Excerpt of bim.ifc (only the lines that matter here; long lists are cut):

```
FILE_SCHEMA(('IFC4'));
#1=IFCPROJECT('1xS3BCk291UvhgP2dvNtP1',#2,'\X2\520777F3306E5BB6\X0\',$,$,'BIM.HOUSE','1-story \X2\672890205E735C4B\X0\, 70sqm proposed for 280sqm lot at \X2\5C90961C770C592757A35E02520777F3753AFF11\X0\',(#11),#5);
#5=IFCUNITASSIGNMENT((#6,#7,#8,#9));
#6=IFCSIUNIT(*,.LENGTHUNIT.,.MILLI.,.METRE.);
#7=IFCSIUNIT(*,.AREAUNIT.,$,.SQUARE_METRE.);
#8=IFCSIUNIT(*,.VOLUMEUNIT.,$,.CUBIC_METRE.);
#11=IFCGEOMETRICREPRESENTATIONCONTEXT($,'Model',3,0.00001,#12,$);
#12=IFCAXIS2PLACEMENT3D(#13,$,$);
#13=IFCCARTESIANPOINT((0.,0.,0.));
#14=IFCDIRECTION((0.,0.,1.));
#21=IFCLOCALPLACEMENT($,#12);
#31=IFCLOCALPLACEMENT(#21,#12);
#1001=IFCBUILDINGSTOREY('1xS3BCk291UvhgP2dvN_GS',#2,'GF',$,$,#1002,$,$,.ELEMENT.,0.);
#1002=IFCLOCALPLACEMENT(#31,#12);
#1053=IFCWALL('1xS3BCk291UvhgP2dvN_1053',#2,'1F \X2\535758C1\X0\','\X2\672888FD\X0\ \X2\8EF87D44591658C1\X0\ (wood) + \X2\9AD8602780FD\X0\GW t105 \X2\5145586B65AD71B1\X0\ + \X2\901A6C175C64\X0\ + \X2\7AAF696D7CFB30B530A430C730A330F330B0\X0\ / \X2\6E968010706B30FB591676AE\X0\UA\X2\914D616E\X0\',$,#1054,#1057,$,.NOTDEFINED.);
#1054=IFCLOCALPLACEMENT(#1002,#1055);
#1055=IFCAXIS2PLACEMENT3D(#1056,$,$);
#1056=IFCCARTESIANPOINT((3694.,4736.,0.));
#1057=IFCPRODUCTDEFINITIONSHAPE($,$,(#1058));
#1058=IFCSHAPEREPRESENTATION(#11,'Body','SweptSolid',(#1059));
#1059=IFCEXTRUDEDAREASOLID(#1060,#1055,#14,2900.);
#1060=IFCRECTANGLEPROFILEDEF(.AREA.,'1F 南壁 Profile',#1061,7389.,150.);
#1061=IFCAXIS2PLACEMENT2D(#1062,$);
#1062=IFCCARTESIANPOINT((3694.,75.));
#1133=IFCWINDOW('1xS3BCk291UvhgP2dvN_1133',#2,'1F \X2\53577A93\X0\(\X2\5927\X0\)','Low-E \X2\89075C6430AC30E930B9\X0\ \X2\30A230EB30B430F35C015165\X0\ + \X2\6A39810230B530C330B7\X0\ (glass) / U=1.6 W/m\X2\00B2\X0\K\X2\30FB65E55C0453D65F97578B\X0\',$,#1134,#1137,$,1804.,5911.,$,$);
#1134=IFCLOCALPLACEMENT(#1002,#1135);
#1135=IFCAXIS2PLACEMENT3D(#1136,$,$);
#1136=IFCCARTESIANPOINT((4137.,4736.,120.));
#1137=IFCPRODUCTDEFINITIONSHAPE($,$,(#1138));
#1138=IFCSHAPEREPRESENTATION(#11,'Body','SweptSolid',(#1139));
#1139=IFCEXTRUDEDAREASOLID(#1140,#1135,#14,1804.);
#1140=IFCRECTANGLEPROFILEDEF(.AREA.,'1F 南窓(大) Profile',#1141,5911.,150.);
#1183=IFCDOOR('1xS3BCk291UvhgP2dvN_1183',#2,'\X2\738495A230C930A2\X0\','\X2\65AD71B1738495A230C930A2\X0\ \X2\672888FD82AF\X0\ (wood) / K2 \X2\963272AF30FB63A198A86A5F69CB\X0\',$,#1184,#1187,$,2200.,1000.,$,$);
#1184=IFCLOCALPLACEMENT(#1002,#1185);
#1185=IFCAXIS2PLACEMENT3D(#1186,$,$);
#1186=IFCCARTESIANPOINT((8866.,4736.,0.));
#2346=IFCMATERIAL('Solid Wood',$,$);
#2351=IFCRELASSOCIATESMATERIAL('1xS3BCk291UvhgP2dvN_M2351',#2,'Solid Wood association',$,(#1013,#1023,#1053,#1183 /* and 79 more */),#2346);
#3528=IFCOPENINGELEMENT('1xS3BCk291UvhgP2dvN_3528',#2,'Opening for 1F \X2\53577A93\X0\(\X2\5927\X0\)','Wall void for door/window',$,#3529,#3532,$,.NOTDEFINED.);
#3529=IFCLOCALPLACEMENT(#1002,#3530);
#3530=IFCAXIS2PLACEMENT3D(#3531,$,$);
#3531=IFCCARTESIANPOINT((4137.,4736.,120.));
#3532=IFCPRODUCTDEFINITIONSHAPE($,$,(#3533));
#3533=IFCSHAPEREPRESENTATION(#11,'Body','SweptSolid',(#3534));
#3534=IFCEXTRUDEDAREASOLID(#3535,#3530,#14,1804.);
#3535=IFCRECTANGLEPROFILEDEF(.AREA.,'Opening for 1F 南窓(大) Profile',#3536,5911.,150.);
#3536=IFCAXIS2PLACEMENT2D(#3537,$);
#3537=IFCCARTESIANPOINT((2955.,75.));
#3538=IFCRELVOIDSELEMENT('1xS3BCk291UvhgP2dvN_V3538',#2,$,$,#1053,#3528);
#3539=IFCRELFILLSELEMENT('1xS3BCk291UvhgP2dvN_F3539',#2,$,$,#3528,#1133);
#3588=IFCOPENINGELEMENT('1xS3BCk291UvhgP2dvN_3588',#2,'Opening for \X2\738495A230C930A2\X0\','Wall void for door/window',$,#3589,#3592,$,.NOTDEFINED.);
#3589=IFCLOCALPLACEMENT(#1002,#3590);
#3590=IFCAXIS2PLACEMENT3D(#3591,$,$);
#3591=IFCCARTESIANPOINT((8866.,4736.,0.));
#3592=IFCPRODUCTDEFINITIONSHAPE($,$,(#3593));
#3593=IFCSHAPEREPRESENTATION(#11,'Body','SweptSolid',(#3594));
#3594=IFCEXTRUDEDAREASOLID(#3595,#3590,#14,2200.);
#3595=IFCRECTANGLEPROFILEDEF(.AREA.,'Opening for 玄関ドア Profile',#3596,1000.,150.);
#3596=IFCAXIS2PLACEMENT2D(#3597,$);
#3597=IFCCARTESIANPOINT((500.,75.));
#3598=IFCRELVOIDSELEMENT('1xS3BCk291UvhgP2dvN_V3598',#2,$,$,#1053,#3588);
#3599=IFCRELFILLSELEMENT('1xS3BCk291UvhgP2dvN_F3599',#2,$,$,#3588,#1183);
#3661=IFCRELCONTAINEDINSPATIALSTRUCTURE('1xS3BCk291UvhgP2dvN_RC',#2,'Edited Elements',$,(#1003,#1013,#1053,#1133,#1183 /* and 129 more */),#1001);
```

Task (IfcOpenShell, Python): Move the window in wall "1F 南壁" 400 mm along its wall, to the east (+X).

```python
import ifcopenshell
import ifcopenshell.api.geometry
import ifcopenshell.util.placement

model = ifcopenshell.open("bim.ifc")

window = model.by_id(1133)
opening = window.FillsVoids[0].RelatingOpeningElement
wall = opening.VoidsElements[0].RelatingBuildingElement

wall_matrix = ifcopenshell.util.placement.get_local_placement(wall.ObjectPlacement)
shift = wall_matrix[:3, 0] * 400.0
before = ifcopenshell.util.placement.get_local_placement(window.ObjectPlacement)[:3, 3].copy()

# The window is not placed relative to its opening, so move both.
for product in (opening, window):
    matrix = ifcopenshell.util.placement.get_local_placement(product.ObjectPlacement)
    matrix[:3, 3] += shift
    ifcopenshell.api.geometry.edit_object_placement(model, product=product, matrix=matrix, is_si=False)

after = ifcopenshell.util.placement.get_local_placement(window.ObjectPlacement)[:3, 3]
print("window moved by", (after - before).round(3) + 0.0)

model.write("bim_updated.ifc")
```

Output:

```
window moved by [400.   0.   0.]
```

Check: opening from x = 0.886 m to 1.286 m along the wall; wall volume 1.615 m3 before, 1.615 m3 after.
